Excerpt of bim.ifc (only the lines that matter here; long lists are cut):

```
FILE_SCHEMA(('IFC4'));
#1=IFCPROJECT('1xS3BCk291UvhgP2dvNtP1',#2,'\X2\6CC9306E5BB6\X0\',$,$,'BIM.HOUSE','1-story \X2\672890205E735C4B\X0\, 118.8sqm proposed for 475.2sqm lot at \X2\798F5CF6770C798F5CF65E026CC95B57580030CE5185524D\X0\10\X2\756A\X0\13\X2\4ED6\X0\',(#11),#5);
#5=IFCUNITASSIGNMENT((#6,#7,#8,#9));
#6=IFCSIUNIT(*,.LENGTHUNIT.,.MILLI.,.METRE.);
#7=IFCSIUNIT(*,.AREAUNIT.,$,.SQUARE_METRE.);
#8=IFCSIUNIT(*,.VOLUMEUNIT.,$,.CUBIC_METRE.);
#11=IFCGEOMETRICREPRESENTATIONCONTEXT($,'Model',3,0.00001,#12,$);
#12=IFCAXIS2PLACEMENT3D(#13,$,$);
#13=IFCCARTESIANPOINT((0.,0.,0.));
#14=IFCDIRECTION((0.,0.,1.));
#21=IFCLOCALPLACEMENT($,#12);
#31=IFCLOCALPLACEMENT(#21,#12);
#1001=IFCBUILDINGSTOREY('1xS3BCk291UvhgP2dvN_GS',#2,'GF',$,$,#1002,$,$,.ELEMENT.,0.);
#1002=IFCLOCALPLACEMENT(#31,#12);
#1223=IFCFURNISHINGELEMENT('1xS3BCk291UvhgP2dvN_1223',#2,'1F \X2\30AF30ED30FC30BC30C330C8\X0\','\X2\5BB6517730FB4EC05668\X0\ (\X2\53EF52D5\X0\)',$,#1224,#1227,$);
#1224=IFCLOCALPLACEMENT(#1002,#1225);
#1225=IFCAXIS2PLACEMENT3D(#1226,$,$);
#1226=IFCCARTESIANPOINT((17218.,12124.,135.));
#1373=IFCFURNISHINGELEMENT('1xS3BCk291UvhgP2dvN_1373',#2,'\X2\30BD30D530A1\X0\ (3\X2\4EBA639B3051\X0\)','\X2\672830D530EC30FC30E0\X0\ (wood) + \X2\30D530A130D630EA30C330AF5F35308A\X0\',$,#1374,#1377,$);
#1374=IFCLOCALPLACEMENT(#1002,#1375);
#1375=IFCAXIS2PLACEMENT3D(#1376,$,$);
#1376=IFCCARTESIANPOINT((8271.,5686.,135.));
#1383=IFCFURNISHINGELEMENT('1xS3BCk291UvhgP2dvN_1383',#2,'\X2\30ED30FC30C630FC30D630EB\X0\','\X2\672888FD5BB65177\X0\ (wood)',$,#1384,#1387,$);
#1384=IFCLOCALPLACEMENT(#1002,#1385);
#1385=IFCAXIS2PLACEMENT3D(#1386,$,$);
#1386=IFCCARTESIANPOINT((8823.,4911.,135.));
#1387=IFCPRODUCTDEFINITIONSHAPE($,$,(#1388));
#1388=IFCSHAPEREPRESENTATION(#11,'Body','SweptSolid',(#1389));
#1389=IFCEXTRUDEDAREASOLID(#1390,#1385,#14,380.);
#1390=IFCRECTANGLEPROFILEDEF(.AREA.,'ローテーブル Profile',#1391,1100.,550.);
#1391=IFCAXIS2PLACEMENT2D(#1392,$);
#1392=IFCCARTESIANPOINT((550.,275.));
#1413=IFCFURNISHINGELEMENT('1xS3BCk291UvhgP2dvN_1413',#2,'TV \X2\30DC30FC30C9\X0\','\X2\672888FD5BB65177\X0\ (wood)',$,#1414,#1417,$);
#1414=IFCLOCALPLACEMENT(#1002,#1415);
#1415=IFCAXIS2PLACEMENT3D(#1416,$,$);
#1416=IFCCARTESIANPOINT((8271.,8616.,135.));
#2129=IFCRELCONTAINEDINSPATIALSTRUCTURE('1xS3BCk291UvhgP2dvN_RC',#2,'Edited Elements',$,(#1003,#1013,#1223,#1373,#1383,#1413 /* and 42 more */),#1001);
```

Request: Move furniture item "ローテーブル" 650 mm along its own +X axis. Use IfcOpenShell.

```python
import ifcopenshell
import ifcopenshell.api.geometry
import ifcopenshell.util.placement
import ifcopenshell.util.unit

model = ifcopenshell.open("bim.ifc")
unit_scale = ifcopenshell.util.unit.calculate_unit_scale(model)

item = model.by_id(1383)
matrix = ifcopenshell.util.placement.get_local_placement(item.ObjectPlacement)
matrix[:3, 3] += matrix[:3, 0] * 0.65 / unit_scale
ifcopenshell.api.geometry.edit_object_placement(model, product=item, matrix=matrix, is_si=False)

print(ifcopenshell.util.placement.get_local_placement(item.ObjectPlacement).round(3) + 0.0)

model.write("bim-out.ifc")
```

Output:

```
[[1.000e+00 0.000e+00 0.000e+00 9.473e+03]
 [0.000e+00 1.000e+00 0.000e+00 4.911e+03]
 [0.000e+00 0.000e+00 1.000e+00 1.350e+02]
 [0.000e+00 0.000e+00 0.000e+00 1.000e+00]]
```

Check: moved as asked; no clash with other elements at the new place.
